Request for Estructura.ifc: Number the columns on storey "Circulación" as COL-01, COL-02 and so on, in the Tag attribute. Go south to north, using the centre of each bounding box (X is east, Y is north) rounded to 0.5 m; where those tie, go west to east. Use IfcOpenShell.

First a look at what the model holds.

```python
import ifcopenshell
import ifcopenshell.util.element
import ifcopenshell.util.placement

model = ifcopenshell.open("Estructura.ifc")
print(model.schema)
storey = next(s for s in model.by_type("IfcBuildingStorey") if s.Name == "Circulación")
columns = [e for e in ifcopenshell.util.element.get_decomposition(storey) if e.is_a("IfcColumn")]
for e in sorted(columns, key=lambda e: e.id()):
    origin = ifcopenshell.util.placement.get_local_placement(e.ObjectPlacement)[:3, 3]
    print(e.id(), e.Tag, e.Name, origin.round(2) + 0.0, sep=" | ")
```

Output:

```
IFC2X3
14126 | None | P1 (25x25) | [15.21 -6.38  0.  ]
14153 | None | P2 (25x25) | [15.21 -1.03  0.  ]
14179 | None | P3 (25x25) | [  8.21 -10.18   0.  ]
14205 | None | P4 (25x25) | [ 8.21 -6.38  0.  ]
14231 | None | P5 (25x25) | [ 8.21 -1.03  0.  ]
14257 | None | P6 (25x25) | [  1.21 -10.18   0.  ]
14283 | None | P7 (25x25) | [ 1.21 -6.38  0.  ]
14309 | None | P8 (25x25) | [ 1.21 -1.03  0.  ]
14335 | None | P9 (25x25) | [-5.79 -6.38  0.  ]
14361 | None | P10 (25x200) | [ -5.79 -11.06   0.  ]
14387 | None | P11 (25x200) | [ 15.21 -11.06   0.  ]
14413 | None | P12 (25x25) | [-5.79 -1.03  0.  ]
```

```python
import ifcopenshell
import ifcopenshell.geom
import ifcopenshell.util.element
import ifcopenshell.util.shape

model = ifcopenshell.open("Estructura.ifc")
settings = ifcopenshell.geom.settings()
settings.set("use-world-coords", True)


def centre(element):
    shape = ifcopenshell.geom.create_shape(settings, element)
    return ifcopenshell.util.shape.get_bbox_centroid(shape.geometry)


storey = next(s for s in model.by_type("IfcBuildingStorey") if s.Name == "Circulación")
columns = [e for e in ifcopenshell.util.element.get_decomposition(storey) if e.is_a("IfcColumn")]

# Insertion points can sit at a corner or the storey origin, so sort by the geometry (in metres).
centres = {e: centre(e) for e in columns}
columns.sort(key=lambda e: (round(centres[e][1] / 0.5), centres[e][0]))

for i, e in enumerate(columns, start=1):
    number = f"COL-{i:02d}"
    e.Tag = number
    print(e.id(), number)

model.write("Estructura-out.ifc")
```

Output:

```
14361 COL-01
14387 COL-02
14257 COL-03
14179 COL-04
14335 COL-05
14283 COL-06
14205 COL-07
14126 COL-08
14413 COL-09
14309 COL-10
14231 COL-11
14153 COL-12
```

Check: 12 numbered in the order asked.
